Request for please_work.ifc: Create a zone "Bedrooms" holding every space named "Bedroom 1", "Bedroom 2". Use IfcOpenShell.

First a look at what the model holds.

```python
import ifcopenshell

model = ifcopenshell.open("please_work.ifc")
print(model.schema)
seen = {}
for space in model.by_type("IfcSpace"):
    seen[space.LongName] = seen.get(space.LongName, 0) + 1
for name, count in sorted(seen.items(), key=str):
    print(count, "x", name)
print("zones:", [z.Name for z in model.by_type("IfcZone")][:20])
```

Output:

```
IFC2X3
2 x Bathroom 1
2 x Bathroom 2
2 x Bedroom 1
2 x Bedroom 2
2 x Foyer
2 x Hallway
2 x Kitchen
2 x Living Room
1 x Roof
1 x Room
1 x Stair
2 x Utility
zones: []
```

```python
import ifcopenshell
import ifcopenshell.api.group
import ifcopenshell.api.root

model = ifcopenshell.open("please_work.ifc")

names = {"Bedroom 1", "Bedroom 2"}
spaces = [s for s in model.by_type("IfcSpace") if s.LongName in names]

zone = ifcopenshell.api.root.create_entity(model, ifc_class="IfcZone", name="Bedrooms")
ifcopenshell.api.group.assign_group(model, products=spaces, group=zone)
print(len(spaces), "spaces in", zone.Name)

model.write("please_work_edited.ifc")
```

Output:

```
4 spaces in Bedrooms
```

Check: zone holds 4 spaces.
